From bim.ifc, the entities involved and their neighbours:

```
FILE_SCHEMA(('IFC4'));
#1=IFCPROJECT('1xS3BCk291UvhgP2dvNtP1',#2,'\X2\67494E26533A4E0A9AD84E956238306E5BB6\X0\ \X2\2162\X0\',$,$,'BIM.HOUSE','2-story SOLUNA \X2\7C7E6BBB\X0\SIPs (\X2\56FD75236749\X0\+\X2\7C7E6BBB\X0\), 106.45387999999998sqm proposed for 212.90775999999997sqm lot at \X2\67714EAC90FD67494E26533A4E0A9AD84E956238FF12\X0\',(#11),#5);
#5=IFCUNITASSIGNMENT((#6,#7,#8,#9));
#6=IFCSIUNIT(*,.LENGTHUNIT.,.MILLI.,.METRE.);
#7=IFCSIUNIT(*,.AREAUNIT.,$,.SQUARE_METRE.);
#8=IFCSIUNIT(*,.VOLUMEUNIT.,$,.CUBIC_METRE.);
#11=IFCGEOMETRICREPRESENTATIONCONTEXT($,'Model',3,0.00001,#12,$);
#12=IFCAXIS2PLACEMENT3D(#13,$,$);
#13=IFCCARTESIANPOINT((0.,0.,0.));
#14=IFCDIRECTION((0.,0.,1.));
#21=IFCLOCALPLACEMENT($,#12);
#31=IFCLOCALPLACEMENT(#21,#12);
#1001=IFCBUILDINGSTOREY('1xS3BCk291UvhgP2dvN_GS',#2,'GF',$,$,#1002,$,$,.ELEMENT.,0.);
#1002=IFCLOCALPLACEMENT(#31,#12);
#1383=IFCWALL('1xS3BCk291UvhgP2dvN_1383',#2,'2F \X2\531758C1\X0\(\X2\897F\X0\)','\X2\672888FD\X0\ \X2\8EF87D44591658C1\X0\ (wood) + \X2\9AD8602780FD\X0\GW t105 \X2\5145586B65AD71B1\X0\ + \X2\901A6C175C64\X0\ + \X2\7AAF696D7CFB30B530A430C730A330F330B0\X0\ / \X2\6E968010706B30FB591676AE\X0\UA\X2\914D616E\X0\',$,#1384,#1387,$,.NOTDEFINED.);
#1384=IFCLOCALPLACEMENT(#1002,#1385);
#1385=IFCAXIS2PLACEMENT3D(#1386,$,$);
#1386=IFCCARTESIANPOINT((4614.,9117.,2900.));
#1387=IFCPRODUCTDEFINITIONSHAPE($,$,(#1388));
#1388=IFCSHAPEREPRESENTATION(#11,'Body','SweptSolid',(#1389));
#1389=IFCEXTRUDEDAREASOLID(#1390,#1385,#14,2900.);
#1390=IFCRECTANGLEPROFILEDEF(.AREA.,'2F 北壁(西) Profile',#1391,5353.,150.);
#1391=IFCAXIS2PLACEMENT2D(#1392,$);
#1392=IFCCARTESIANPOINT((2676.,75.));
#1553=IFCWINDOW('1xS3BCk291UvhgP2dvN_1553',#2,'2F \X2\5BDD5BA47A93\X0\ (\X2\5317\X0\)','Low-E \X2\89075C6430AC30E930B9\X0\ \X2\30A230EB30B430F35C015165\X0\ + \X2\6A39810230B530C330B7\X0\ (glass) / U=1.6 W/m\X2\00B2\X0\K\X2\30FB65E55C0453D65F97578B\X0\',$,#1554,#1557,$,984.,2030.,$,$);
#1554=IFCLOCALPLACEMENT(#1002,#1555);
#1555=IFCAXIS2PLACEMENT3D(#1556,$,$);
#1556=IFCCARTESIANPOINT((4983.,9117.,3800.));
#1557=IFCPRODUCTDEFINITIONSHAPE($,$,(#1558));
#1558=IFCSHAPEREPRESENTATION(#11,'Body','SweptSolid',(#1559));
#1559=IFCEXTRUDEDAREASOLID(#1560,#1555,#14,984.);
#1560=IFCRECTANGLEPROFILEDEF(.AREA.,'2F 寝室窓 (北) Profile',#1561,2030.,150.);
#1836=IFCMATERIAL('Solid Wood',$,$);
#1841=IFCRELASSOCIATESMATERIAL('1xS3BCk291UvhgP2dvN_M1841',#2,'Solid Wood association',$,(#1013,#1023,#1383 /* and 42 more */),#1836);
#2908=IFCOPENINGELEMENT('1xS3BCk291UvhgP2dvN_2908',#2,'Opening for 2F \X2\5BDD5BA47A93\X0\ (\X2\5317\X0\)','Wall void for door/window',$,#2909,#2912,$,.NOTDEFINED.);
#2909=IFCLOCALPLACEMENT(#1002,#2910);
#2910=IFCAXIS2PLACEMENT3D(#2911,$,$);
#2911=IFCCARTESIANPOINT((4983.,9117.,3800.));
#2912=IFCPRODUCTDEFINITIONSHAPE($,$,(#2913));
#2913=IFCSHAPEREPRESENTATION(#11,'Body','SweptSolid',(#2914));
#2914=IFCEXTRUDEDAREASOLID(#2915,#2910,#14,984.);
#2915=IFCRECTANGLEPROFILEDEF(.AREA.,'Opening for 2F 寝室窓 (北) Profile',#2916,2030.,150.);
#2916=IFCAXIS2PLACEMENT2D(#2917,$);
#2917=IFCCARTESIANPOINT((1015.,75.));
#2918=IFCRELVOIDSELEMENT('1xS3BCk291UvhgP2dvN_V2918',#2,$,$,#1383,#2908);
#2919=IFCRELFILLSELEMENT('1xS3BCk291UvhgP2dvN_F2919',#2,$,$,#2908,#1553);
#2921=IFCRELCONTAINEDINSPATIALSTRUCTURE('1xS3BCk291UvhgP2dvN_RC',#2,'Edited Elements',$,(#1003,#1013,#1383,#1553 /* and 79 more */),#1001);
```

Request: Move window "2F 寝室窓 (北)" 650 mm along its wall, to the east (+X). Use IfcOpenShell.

```python
import ifcopenshell
import ifcopenshell.api.geometry
import ifcopenshell.util.placement

model = ifcopenshell.open("bim.ifc")

window = model.by_guid("1xS3BCk291UvhgP2dvN_1553")
opening = window.FillsVoids[0].RelatingOpeningElement
wall = opening.VoidsElements[0].RelatingBuildingElement

wall_matrix = ifcopenshell.util.placement.get_local_placement(wall.ObjectPlacement)
shift = wall_matrix[:3, 0] * 650.0
before = ifcopenshell.util.placement.get_local_placement(window.ObjectPlacement)[:3, 3].copy()

# The window is not placed relative to its opening, so move both.
for product in (opening, window):
    matrix = ifcopenshell.util.placement.get_local_placement(product.ObjectPlacement)
    matrix[:3, 3] += shift
    ifcopenshell.api.geometry.edit_object_placement(model, product=product, matrix=matrix, is_si=False)

after = ifcopenshell.util.placement.get_local_placement(window.ObjectPlacement)[:3, 3]
print("window moved by", (after - before).round(3) + 0.0)

model.write("bim-out.ifc")
```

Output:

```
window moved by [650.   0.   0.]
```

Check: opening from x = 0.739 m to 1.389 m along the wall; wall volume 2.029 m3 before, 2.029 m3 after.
